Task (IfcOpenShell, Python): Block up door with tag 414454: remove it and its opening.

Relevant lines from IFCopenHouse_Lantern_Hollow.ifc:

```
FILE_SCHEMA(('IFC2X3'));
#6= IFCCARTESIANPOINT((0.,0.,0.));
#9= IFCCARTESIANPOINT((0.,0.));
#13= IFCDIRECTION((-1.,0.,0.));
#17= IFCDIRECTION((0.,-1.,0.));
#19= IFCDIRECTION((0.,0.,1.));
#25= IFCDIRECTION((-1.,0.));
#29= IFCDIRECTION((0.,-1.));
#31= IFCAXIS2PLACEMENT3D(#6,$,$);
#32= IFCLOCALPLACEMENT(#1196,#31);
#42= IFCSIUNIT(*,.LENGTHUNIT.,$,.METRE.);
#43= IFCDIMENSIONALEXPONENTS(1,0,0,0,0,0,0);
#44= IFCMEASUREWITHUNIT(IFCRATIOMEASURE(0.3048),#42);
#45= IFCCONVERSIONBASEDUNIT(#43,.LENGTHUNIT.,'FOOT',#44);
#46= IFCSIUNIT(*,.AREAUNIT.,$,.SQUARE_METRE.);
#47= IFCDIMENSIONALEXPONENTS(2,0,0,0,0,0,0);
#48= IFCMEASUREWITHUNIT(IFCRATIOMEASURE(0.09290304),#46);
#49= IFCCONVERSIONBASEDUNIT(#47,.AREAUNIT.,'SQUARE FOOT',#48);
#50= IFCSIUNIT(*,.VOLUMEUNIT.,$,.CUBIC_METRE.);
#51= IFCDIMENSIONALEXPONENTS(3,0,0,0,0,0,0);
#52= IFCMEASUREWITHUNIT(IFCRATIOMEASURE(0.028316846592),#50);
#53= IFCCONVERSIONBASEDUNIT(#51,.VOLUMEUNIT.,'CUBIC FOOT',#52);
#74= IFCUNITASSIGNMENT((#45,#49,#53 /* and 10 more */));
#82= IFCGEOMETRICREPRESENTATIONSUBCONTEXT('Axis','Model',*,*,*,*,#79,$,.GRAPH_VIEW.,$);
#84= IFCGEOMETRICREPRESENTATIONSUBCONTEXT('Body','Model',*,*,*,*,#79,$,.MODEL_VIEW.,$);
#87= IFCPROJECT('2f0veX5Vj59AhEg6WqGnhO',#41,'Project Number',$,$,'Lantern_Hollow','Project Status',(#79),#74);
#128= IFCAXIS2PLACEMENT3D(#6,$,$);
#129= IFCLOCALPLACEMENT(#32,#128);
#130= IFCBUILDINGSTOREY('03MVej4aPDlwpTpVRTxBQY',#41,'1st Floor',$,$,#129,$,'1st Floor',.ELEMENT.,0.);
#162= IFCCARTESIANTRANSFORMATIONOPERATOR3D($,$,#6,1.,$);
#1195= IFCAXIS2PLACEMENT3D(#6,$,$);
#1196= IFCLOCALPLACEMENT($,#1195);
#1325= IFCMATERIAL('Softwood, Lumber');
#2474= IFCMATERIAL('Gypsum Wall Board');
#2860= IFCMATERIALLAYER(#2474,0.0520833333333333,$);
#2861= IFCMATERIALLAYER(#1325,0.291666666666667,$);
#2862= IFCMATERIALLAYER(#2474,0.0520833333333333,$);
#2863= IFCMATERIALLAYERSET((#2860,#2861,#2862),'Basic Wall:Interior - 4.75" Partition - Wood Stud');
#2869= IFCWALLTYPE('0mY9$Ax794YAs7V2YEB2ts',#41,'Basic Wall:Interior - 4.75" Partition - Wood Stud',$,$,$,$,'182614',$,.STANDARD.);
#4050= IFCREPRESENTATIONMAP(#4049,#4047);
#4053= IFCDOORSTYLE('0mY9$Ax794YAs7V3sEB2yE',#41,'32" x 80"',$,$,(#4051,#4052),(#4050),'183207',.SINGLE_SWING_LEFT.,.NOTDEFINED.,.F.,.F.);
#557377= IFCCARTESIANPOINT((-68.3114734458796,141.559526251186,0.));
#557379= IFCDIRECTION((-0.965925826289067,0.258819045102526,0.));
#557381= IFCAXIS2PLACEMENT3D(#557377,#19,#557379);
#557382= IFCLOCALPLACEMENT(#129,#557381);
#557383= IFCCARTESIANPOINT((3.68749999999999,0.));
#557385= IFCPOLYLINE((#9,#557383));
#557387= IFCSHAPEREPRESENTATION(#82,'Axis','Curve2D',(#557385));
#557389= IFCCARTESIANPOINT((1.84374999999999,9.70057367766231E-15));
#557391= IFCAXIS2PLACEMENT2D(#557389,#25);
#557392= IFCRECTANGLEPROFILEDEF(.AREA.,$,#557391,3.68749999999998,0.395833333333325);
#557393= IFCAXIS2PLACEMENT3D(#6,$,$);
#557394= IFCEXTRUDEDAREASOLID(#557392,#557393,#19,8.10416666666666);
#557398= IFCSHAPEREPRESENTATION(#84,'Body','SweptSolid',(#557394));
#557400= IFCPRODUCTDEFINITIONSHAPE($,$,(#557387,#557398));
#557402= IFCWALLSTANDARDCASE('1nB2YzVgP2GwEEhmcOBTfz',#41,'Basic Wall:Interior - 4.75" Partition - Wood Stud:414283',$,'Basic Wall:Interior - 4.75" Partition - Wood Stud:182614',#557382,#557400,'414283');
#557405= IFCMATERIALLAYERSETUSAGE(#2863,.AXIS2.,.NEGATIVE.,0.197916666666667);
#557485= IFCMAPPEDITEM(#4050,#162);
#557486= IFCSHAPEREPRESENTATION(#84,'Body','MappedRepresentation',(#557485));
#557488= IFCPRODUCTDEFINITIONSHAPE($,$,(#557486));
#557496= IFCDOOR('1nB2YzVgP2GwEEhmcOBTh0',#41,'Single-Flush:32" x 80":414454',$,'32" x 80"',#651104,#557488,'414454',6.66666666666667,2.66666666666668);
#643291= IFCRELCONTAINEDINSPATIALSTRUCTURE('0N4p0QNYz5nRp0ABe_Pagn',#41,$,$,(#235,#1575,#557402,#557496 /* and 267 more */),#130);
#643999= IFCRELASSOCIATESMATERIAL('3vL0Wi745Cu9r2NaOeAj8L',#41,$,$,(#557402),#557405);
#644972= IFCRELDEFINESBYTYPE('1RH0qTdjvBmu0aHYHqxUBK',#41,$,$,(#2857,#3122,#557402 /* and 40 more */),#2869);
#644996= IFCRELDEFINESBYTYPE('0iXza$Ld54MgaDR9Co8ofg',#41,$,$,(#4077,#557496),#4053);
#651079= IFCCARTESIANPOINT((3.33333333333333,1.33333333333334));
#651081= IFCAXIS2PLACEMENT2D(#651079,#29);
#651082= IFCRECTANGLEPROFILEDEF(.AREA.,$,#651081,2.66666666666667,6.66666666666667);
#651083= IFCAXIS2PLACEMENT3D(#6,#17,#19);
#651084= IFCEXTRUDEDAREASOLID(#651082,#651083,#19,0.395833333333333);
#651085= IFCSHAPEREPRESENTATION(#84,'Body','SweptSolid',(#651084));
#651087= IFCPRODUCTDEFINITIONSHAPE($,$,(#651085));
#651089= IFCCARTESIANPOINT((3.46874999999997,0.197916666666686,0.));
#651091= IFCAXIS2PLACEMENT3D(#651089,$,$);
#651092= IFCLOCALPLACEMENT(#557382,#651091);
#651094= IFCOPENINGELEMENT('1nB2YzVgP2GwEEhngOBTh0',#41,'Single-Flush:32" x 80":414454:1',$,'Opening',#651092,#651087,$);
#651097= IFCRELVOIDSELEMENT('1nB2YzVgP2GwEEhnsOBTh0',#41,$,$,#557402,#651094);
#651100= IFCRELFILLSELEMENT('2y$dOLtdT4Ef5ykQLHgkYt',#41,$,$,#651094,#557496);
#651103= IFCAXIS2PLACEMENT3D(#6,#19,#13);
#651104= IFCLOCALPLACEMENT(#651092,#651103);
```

```python
import ifcopenshell
import ifcopenshell.api.feature
import ifcopenshell.api.root
import ifcopenshell.geom
import ifcopenshell.util.shape

model = ifcopenshell.open("IFCopenHouse_Lantern_Hollow.ifc")
settings = ifcopenshell.geom.settings()


def volume(element):
    """Net volume in cubic metres, openings subtracted."""
    shape = ifcopenshell.geom.create_shape(settings, element)
    return ifcopenshell.util.shape.get_volume(shape.geometry)


door = model.by_guid("1nB2YzVgP2GwEEhmcOBTh0")
opening = door.FillsVoids[0].RelatingOpeningElement
wall = opening.VoidsElements[0].RelatingBuildingElement
before = volume(wall)

ifcopenshell.api.root.remove_product(model, product=door)
ifcopenshell.api.feature.remove_feature(model, feature=opening)

after = volume(wall)

print(f"wall volume {before:.3f} -> {after:.3f} m3")

model.write("IFCopenHouse_Lantern_Hollow_rev.ifc")
```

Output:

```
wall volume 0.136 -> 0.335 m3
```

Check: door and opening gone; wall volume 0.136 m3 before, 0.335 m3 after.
